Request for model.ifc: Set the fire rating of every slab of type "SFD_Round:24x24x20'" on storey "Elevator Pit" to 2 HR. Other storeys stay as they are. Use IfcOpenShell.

First a look at what the model holds.

```python
import ifcopenshell
import ifcopenshell.util.element

model = ifcopenshell.open("model.ifc")
print(model.schema)
storey = next(s for s in model.by_type("IfcBuildingStorey") if s.Name == "Elevator Pit")
slabs = [e for e in ifcopenshell.util.element.get_decomposition(storey) if e.is_a("IfcSlab")]
seen = {}
for e in slabs:
    element_type = ifcopenshell.util.element.get_type(e)
    key = (element_type.Name if element_type != e and element_type else None, ifcopenshell.util.element.get_pset(e, "Pset_SlabCommon", "FireRating"))
    seen[key] = seen.get(key, 0) + 1
for (name, value), count in sorted(seen.items(), key=str):
    print(count, "x", name, "|", value)
```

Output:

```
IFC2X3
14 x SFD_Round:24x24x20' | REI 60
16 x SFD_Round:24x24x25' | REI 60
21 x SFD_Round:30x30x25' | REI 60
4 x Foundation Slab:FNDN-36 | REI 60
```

```python
import ifcopenshell
import ifcopenshell.api.pset
import ifcopenshell.util.element

model = ifcopenshell.open("model.ifc")

storey = next(s for s in model.by_type("IfcBuildingStorey") if s.Name == "Elevator Pit")
slabs = [e for e in ifcopenshell.util.element.get_decomposition(storey) if e.is_a("IfcSlab")]

count = 0
for e in slabs:
    element_type = ifcopenshell.util.element.get_type(e)
    if element_type in (None, e) or element_type.Name != "SFD_Round:24x24x20'":
        continue
    # add_pset returns the element's existing set when there is one.
    pset = ifcopenshell.api.pset.add_pset(model, product=e, name="Pset_SlabCommon")
    ifcopenshell.api.pset.edit_pset(model, pset=pset, properties={"FireRating": "2 HR"})
    count += 1

print(count, "slabs updated")

model.write("model_rev.ifc")
```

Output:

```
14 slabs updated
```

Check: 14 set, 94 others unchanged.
